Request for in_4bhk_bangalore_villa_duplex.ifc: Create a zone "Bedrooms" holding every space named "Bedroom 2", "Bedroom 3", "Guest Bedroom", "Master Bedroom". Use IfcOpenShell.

First a look at what the model holds.

```python
import ifcopenshell

model = ifcopenshell.open("in_4bhk_bangalore_villa_duplex.ifc")
print(model.schema)
seen = {}
for space in model.by_type("IfcSpace"):
    seen[space.LongName] = seen.get(space.LongName, 0) + 1
for name, count in sorted(seen.items(), key=str):
    print(count, "x", name)
print("zones:", [z.Name for z in model.by_type("IfcZone")][:20])
```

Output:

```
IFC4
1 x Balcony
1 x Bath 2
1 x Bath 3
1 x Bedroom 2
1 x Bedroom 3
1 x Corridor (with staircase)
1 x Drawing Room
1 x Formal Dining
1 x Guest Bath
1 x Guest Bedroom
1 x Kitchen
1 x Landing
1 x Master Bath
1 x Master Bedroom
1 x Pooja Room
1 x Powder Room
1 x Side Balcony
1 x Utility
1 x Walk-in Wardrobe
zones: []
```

```python
import ifcopenshell
import ifcopenshell.api.group
import ifcopenshell.api.root

model = ifcopenshell.open("in_4bhk_bangalore_villa_duplex.ifc")

names = {"Bedroom 2", "Bedroom 3", "Guest Bedroom", "Master Bedroom"}
spaces = [s for s in model.by_type("IfcSpace") if s.LongName in names]

zone = ifcopenshell.api.root.create_entity(model, ifc_class="IfcZone", name="Bedrooms")
ifcopenshell.api.group.assign_group(model, products=spaces, group=zone)
print(len(spaces), "spaces in", zone.Name)

model.write("in_4bhk_bangalore_villa_duplex_updated.ifc")
```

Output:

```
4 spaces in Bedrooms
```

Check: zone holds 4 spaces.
